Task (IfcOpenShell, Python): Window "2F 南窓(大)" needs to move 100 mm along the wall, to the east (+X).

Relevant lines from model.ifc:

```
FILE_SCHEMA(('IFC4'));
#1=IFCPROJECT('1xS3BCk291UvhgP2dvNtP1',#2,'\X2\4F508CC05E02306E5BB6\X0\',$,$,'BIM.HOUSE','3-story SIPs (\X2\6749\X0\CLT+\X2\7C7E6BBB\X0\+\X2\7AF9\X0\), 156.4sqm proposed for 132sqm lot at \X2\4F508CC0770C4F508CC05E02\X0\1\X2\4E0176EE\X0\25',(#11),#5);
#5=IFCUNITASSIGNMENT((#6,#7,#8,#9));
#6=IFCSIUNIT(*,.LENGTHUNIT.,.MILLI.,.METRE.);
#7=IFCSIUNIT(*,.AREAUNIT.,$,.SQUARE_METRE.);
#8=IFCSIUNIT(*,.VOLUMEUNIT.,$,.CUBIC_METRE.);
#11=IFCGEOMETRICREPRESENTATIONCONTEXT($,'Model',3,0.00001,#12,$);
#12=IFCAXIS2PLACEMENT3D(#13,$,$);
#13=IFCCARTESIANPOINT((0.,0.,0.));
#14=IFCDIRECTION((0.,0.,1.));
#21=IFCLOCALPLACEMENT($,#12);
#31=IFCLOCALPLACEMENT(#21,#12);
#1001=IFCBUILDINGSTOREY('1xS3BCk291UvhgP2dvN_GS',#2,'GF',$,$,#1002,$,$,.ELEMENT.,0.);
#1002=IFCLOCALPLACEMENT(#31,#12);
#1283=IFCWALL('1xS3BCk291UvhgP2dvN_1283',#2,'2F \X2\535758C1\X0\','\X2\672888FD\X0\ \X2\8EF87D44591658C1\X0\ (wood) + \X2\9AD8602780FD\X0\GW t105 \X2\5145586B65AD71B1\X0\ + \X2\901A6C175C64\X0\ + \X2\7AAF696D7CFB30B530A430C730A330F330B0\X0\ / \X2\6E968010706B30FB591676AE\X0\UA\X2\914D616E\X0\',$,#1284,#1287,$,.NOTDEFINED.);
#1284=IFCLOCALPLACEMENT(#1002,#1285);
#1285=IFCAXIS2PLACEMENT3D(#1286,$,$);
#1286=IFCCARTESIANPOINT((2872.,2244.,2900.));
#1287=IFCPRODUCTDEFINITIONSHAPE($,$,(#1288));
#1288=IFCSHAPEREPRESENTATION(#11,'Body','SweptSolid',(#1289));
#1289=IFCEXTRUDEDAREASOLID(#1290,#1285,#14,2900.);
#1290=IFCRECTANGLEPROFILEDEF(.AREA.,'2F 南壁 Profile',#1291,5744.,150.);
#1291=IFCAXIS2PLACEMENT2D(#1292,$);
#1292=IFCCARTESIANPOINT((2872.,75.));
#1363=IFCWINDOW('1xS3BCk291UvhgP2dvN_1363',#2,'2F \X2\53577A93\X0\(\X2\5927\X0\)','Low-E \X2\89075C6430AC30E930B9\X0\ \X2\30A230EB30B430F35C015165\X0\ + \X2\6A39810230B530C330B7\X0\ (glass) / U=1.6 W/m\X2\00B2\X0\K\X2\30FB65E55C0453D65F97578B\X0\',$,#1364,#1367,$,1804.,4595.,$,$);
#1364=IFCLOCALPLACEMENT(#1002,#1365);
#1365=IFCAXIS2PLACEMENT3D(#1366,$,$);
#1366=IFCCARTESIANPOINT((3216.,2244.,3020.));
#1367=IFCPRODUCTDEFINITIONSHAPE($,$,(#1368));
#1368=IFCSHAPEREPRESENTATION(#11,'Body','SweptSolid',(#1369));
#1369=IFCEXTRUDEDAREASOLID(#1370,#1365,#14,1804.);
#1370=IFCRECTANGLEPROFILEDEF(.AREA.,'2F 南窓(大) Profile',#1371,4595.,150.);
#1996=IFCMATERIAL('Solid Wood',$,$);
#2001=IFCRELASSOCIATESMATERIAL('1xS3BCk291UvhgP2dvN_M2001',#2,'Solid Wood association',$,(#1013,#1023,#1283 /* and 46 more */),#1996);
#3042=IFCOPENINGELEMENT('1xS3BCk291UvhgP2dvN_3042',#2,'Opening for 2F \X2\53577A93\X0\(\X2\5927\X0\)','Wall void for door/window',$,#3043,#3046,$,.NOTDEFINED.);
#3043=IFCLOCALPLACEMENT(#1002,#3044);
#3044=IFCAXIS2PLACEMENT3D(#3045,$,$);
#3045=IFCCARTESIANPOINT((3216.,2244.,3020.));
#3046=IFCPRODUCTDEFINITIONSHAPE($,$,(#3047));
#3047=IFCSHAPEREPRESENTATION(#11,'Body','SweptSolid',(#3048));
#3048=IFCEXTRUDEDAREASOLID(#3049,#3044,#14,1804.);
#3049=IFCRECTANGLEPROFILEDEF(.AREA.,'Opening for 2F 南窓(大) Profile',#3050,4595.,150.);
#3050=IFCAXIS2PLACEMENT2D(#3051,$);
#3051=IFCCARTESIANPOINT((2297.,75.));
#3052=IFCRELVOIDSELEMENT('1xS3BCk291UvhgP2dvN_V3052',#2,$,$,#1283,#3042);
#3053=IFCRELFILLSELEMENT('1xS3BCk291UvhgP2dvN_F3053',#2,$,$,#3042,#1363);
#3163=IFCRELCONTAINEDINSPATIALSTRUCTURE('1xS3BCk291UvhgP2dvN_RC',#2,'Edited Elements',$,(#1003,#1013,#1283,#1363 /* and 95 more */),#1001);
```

```python
import ifcopenshell
import ifcopenshell.api.geometry
import ifcopenshell.util.placement
import ifcopenshell.util.unit

model = ifcopenshell.open("model.ifc")
unit_scale = ifcopenshell.util.unit.calculate_unit_scale(model)

window = model.by_id(1363)
opening = window.FillsVoids[0].RelatingOpeningElement
wall = opening.VoidsElements[0].RelatingBuildingElement

wall_matrix = ifcopenshell.util.placement.get_local_placement(wall.ObjectPlacement)
shift = wall_matrix[:3, 0] * 0.1 / unit_scale
before = ifcopenshell.util.placement.get_local_placement(window.ObjectPlacement)[:3, 3].copy()

# The window is not placed relative to its opening, so move both.
for product in (opening, window):
    matrix = ifcopenshell.util.placement.get_local_placement(product.ObjectPlacement)
    matrix[:3, 3] += shift
    ifcopenshell.api.geometry.edit_object_placement(model, product=product, matrix=matrix, is_si=False)

after = ifcopenshell.util.placement.get_local_placement(window.ObjectPlacement)[:3, 3]
print("window moved by", (after - before).round(3) + 0.0)

model.write("model_updated.ifc")
```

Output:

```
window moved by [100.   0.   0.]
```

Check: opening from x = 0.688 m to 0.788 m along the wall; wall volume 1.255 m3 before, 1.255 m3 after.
